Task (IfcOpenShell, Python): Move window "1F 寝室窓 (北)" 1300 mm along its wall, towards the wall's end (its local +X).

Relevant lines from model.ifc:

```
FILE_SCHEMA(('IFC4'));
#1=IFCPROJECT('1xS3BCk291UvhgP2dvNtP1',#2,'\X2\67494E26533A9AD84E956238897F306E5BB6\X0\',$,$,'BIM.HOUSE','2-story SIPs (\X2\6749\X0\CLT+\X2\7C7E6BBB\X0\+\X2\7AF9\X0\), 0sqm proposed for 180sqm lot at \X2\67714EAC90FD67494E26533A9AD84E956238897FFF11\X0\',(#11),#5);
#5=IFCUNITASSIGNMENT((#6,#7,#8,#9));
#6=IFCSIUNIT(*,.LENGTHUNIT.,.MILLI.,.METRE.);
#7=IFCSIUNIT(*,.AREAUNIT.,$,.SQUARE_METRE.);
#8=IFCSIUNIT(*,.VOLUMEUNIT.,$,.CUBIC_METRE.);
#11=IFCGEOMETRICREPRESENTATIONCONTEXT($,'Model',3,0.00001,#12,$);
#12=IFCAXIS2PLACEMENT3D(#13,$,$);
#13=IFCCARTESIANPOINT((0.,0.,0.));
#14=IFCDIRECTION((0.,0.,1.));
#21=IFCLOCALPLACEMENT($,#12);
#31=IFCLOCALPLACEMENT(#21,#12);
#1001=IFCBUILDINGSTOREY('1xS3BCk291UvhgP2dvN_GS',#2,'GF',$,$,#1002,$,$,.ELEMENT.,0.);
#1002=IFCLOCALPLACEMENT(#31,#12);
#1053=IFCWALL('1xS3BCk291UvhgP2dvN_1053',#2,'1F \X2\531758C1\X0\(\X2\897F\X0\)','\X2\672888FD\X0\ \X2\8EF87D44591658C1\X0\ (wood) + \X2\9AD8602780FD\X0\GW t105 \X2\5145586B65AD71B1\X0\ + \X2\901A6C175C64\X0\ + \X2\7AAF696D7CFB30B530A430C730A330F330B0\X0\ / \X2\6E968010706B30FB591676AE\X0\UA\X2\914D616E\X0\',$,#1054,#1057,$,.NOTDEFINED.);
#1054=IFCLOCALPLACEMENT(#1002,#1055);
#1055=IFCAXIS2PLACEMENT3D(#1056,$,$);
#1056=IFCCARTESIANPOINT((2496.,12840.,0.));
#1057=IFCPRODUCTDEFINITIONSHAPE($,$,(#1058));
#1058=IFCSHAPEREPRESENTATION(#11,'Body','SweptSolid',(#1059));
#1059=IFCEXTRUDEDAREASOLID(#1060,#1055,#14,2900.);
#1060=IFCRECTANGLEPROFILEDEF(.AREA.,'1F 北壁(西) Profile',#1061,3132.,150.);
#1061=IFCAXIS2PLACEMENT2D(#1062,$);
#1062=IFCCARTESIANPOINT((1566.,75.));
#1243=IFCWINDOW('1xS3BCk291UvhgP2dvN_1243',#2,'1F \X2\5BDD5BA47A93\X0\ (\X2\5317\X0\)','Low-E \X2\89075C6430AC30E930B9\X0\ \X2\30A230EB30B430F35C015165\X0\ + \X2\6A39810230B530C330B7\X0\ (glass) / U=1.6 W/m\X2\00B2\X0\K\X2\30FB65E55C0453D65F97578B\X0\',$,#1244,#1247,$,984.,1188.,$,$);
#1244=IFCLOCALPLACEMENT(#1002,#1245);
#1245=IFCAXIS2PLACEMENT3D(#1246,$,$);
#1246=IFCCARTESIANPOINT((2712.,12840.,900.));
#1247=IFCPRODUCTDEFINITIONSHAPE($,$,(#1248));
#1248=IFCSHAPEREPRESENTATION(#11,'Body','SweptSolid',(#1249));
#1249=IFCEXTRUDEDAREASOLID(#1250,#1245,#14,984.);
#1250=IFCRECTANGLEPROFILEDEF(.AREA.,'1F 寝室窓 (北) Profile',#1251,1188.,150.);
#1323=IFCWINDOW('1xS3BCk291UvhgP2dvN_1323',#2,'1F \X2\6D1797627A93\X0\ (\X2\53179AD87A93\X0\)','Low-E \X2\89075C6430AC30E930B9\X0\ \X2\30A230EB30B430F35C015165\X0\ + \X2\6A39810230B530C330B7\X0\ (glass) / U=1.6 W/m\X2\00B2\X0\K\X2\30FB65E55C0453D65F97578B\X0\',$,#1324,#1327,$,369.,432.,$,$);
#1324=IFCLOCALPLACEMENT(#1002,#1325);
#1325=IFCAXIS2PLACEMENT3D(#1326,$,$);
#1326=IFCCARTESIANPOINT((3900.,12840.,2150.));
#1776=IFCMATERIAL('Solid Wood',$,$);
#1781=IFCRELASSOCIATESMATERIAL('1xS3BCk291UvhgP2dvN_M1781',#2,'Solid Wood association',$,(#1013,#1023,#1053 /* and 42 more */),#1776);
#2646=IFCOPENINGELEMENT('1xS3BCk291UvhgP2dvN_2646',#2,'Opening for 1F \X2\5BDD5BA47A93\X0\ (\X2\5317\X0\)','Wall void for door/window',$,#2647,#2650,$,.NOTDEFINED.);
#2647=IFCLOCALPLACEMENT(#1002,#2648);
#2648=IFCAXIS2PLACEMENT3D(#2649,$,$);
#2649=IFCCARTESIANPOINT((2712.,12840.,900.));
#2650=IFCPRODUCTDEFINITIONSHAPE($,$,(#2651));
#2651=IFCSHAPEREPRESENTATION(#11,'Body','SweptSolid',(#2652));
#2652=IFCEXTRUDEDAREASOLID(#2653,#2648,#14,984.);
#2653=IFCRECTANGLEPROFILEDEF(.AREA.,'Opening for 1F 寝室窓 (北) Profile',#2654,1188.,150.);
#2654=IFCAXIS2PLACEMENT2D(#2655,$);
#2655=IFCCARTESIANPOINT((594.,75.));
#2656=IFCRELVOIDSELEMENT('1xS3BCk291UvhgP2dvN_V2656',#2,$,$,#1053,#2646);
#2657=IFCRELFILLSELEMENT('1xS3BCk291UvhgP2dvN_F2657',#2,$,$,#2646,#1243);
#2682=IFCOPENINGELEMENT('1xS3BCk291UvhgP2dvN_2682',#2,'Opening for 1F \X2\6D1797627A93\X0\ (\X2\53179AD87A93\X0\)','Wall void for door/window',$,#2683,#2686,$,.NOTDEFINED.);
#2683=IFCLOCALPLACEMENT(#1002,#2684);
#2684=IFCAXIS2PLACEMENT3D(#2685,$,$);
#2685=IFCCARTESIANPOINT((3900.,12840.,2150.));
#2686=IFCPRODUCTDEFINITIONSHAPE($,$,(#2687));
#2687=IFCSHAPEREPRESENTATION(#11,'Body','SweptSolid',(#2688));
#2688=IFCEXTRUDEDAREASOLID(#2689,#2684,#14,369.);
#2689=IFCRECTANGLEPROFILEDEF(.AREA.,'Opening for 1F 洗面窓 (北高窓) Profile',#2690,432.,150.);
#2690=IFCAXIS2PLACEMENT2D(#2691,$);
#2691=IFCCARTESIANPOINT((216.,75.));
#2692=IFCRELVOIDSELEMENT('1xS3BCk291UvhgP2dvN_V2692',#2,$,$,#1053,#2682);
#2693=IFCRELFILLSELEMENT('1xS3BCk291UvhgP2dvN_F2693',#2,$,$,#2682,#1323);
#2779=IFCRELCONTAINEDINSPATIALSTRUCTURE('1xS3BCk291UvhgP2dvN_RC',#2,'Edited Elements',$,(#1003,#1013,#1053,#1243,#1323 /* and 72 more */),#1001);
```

```python
import ifcopenshell
import ifcopenshell.api.geometry
import ifcopenshell.util.placement

model = ifcopenshell.open("model.ifc")

window = model.by_guid("1xS3BCk291UvhgP2dvN_1243")
opening = window.FillsVoids[0].RelatingOpeningElement
wall = opening.VoidsElements[0].RelatingBuildingElement

wall_matrix = ifcopenshell.util.placement.get_local_placement(wall.ObjectPlacement)
shift = wall_matrix[:3, 0] * 1300.0
before = ifcopenshell.util.placement.get_local_placement(window.ObjectPlacement)[:3, 3].copy()

# The window is not placed relative to its opening, so move both.
for product in (opening, window):
    matrix = ifcopenshell.util.placement.get_local_placement(product.ObjectPlacement)
    matrix[:3, 3] += shift
    ifcopenshell.api.geometry.edit_object_placement(model, product=product, matrix=matrix, is_si=False)

after = ifcopenshell.util.placement.get_local_placement(window.ObjectPlacement)[:3, 3]
print("window moved by", (after - before).round(3) + 0.0)

model.write("model-out.ifc")
```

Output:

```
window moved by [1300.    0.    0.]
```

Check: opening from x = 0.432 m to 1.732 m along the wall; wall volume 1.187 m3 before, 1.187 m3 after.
